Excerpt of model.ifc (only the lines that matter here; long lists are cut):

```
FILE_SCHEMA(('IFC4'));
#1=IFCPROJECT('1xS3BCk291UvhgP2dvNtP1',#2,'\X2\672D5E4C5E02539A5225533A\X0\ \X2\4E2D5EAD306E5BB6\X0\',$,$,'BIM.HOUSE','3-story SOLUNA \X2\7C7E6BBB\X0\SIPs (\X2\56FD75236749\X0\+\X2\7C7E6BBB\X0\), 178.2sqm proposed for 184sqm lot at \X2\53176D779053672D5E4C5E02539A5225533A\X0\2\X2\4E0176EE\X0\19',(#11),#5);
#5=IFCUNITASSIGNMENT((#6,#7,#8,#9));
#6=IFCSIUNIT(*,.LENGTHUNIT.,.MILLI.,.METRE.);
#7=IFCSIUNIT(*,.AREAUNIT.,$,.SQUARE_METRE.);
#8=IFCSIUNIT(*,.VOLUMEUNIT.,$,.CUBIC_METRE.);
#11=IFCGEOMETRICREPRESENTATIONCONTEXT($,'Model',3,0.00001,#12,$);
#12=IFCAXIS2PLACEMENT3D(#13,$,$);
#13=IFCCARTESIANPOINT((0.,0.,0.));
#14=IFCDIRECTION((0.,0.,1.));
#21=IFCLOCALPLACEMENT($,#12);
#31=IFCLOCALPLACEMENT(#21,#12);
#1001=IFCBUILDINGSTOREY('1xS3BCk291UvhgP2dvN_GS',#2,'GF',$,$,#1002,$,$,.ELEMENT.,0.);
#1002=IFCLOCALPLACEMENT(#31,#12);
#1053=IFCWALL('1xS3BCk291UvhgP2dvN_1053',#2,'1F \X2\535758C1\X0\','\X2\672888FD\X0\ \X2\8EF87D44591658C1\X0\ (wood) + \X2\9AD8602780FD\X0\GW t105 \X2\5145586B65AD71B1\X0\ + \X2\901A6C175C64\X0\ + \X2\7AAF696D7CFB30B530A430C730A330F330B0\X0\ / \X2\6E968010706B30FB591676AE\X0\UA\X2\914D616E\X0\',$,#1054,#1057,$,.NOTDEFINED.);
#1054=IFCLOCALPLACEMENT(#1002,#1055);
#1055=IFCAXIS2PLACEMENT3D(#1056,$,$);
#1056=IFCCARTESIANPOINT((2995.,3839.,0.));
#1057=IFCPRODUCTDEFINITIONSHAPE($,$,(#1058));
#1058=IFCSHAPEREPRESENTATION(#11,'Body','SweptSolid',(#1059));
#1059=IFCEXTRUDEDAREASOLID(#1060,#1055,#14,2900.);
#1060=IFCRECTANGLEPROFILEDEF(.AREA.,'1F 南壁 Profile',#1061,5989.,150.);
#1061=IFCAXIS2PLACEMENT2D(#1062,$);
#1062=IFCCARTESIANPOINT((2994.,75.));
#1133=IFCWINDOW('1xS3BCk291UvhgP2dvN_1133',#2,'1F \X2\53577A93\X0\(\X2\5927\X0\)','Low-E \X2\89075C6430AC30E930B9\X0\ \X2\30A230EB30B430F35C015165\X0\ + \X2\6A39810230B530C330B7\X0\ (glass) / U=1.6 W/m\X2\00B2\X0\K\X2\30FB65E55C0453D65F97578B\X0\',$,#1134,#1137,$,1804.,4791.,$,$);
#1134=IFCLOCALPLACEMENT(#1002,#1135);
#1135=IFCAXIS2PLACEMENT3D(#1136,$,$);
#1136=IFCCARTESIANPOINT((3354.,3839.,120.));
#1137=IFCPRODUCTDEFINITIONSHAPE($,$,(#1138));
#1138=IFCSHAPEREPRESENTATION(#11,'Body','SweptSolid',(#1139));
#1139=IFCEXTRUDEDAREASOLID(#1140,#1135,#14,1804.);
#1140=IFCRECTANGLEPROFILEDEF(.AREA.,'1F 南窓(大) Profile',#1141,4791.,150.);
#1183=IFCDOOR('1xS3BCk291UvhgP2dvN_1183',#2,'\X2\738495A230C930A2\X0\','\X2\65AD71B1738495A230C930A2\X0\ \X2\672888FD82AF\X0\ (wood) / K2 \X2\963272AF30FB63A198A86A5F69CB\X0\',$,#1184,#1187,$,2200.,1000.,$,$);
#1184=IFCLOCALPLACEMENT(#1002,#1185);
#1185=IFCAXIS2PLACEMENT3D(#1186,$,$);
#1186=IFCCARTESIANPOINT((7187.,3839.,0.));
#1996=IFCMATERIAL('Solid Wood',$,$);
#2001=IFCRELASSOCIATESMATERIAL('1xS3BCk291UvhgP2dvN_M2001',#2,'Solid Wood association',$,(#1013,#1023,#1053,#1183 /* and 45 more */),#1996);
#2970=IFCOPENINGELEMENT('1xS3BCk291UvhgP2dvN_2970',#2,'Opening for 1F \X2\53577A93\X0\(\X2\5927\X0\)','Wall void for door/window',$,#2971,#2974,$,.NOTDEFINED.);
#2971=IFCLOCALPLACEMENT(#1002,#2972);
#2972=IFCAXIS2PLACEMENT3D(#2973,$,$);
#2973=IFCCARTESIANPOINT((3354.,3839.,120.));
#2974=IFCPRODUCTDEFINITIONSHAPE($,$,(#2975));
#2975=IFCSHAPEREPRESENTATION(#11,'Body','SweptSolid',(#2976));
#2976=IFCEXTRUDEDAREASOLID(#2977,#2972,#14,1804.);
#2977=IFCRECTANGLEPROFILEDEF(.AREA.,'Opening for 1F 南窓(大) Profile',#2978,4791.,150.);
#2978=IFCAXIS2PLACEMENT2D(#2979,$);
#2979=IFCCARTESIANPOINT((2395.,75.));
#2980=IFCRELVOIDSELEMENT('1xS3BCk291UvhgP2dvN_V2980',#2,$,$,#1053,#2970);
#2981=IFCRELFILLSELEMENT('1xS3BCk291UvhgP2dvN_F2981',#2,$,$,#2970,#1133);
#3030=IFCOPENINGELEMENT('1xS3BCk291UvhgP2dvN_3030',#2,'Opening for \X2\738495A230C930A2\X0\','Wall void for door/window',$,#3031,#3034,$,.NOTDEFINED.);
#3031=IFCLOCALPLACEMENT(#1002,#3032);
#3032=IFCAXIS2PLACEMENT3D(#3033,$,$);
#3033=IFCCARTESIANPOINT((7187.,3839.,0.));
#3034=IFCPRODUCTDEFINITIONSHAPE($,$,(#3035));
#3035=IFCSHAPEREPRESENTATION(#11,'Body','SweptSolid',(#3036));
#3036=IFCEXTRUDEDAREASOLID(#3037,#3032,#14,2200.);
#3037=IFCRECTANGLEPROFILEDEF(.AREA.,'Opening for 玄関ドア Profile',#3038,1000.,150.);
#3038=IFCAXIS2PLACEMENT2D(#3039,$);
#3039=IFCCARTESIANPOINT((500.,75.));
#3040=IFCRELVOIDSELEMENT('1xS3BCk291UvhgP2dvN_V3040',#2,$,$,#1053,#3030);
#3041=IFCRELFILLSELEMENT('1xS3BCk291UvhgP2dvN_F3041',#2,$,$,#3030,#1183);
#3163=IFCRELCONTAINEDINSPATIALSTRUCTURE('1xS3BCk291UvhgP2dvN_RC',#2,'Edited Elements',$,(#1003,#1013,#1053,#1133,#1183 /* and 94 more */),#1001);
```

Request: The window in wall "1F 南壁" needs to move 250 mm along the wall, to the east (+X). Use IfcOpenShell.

```python
import ifcopenshell
import ifcopenshell.api.geometry
import ifcopenshell.util.placement
import ifcopenshell.util.unit

model = ifcopenshell.open("model.ifc")
unit_scale = ifcopenshell.util.unit.calculate_unit_scale(model)

window = model.by_guid("1xS3BCk291UvhgP2dvN_1133")
opening = window.FillsVoids[0].RelatingOpeningElement
wall = opening.VoidsElements[0].RelatingBuildingElement

wall_matrix = ifcopenshell.util.placement.get_local_placement(wall.ObjectPlacement)
shift = wall_matrix[:3, 0] * 0.25 / unit_scale
before = ifcopenshell.util.placement.get_local_placement(window.ObjectPlacement)[:3, 3].copy()

# The window is not placed relative to its opening, so move both.
for product in (opening, window):
    matrix = ifcopenshell.util.placement.get_local_placement(product.ObjectPlacement)
    matrix[:3, 3] += shift
    ifcopenshell.api.geometry.edit_object_placement(model, product=product, matrix=matrix, is_si=False)

after = ifcopenshell.util.placement.get_local_placement(window.ObjectPlacement)[:3, 3]
print("window moved by", (after - before).round(3) + 0.0)

model.write("model_rev.ifc")
```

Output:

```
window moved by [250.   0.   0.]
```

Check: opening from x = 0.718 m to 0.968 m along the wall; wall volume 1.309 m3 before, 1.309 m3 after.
